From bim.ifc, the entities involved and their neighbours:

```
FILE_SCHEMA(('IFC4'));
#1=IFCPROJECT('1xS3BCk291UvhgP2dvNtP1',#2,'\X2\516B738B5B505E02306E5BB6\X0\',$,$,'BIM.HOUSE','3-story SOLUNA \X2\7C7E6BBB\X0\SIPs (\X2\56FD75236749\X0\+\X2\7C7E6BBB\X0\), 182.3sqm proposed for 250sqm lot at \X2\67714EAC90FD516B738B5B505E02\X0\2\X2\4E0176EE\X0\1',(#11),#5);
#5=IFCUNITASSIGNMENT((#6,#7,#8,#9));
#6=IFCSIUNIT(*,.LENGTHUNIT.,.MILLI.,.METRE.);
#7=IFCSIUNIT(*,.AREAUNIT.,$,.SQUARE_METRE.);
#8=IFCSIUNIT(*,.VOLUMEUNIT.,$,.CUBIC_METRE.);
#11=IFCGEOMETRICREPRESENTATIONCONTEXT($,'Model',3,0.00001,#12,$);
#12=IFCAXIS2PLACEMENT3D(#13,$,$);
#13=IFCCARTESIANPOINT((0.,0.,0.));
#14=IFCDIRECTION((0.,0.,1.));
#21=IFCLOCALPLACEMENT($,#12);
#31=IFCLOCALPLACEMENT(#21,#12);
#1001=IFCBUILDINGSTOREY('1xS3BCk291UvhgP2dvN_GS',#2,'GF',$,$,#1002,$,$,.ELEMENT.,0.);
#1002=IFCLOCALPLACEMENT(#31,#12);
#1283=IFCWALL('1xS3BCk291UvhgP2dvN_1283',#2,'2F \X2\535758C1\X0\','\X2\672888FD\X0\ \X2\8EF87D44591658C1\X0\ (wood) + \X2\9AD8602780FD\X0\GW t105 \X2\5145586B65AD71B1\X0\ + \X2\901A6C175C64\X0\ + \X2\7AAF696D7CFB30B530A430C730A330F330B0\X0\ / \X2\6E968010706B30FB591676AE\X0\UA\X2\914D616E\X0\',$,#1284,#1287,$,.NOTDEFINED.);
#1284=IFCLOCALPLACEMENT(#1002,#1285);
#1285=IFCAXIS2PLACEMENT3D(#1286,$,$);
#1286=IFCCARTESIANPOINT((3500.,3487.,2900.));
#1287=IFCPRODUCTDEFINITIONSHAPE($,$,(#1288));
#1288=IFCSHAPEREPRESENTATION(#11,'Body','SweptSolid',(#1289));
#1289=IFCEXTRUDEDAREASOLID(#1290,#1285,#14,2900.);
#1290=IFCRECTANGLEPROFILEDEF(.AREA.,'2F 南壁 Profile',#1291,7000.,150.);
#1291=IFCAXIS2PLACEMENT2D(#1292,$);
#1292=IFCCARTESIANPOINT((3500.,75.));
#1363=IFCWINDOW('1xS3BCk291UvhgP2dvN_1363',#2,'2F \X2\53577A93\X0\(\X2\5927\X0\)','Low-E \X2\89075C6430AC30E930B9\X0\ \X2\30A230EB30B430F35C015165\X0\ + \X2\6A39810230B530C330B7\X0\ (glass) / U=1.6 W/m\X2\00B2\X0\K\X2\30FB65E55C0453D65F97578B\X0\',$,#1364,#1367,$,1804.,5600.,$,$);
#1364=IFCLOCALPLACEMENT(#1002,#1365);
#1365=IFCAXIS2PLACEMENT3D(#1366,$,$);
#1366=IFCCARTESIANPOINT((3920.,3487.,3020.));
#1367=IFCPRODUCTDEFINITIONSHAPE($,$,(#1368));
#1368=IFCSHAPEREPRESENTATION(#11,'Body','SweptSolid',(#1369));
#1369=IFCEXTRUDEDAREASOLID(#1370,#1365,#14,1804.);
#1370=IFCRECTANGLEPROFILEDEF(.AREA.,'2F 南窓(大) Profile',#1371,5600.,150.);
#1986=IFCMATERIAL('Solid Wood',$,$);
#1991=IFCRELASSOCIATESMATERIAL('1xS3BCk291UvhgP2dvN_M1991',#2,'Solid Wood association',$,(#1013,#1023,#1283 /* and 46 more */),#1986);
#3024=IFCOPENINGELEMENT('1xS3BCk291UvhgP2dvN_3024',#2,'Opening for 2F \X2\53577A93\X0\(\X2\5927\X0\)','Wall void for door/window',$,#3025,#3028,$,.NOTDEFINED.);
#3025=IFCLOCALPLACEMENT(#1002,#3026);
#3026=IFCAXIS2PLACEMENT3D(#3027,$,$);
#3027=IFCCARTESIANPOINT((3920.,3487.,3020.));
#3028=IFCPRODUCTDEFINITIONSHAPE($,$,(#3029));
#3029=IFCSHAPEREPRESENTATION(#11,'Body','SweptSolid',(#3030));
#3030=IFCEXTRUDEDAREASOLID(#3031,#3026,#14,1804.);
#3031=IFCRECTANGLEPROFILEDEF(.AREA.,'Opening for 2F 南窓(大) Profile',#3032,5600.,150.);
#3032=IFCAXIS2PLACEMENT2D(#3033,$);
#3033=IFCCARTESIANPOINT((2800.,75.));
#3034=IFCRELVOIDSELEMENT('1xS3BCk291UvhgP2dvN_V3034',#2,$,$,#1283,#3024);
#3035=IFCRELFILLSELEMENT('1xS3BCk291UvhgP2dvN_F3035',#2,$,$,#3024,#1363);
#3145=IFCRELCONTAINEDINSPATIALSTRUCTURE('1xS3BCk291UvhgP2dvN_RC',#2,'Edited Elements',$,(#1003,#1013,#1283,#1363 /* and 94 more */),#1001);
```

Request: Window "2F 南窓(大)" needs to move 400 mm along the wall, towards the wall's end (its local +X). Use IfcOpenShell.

```python
import ifcopenshell
import ifcopenshell.api.geometry
import ifcopenshell.util.placement
import ifcopenshell.util.unit

model = ifcopenshell.open("bim.ifc")
unit_scale = ifcopenshell.util.unit.calculate_unit_scale(model)

window = model.by_guid("1xS3BCk291UvhgP2dvN_1363")
opening = window.FillsVoids[0].RelatingOpeningElement
wall = opening.VoidsElements[0].RelatingBuildingElement

wall_matrix = ifcopenshell.util.placement.get_local_placement(wall.ObjectPlacement)
shift = wall_matrix[:3, 0] * 0.4 / unit_scale
before = ifcopenshell.util.placement.get_local_placement(window.ObjectPlacement)[:3, 3].copy()

# The window is not placed relative to its opening, so move both.
for product in (opening, window):
    matrix = ifcopenshell.util.placement.get_local_placement(product.ObjectPlacement)
    matrix[:3, 3] += shift
    ifcopenshell.api.geometry.edit_object_placement(model, product=product, matrix=matrix, is_si=False)

after = ifcopenshell.util.placement.get_local_placement(window.ObjectPlacement)[:3, 3]
print("window moved by", (after - before).round(3) + 0.0)

model.write("bim_v2.ifc")
```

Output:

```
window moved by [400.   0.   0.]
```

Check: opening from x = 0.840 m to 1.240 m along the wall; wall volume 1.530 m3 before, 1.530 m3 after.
